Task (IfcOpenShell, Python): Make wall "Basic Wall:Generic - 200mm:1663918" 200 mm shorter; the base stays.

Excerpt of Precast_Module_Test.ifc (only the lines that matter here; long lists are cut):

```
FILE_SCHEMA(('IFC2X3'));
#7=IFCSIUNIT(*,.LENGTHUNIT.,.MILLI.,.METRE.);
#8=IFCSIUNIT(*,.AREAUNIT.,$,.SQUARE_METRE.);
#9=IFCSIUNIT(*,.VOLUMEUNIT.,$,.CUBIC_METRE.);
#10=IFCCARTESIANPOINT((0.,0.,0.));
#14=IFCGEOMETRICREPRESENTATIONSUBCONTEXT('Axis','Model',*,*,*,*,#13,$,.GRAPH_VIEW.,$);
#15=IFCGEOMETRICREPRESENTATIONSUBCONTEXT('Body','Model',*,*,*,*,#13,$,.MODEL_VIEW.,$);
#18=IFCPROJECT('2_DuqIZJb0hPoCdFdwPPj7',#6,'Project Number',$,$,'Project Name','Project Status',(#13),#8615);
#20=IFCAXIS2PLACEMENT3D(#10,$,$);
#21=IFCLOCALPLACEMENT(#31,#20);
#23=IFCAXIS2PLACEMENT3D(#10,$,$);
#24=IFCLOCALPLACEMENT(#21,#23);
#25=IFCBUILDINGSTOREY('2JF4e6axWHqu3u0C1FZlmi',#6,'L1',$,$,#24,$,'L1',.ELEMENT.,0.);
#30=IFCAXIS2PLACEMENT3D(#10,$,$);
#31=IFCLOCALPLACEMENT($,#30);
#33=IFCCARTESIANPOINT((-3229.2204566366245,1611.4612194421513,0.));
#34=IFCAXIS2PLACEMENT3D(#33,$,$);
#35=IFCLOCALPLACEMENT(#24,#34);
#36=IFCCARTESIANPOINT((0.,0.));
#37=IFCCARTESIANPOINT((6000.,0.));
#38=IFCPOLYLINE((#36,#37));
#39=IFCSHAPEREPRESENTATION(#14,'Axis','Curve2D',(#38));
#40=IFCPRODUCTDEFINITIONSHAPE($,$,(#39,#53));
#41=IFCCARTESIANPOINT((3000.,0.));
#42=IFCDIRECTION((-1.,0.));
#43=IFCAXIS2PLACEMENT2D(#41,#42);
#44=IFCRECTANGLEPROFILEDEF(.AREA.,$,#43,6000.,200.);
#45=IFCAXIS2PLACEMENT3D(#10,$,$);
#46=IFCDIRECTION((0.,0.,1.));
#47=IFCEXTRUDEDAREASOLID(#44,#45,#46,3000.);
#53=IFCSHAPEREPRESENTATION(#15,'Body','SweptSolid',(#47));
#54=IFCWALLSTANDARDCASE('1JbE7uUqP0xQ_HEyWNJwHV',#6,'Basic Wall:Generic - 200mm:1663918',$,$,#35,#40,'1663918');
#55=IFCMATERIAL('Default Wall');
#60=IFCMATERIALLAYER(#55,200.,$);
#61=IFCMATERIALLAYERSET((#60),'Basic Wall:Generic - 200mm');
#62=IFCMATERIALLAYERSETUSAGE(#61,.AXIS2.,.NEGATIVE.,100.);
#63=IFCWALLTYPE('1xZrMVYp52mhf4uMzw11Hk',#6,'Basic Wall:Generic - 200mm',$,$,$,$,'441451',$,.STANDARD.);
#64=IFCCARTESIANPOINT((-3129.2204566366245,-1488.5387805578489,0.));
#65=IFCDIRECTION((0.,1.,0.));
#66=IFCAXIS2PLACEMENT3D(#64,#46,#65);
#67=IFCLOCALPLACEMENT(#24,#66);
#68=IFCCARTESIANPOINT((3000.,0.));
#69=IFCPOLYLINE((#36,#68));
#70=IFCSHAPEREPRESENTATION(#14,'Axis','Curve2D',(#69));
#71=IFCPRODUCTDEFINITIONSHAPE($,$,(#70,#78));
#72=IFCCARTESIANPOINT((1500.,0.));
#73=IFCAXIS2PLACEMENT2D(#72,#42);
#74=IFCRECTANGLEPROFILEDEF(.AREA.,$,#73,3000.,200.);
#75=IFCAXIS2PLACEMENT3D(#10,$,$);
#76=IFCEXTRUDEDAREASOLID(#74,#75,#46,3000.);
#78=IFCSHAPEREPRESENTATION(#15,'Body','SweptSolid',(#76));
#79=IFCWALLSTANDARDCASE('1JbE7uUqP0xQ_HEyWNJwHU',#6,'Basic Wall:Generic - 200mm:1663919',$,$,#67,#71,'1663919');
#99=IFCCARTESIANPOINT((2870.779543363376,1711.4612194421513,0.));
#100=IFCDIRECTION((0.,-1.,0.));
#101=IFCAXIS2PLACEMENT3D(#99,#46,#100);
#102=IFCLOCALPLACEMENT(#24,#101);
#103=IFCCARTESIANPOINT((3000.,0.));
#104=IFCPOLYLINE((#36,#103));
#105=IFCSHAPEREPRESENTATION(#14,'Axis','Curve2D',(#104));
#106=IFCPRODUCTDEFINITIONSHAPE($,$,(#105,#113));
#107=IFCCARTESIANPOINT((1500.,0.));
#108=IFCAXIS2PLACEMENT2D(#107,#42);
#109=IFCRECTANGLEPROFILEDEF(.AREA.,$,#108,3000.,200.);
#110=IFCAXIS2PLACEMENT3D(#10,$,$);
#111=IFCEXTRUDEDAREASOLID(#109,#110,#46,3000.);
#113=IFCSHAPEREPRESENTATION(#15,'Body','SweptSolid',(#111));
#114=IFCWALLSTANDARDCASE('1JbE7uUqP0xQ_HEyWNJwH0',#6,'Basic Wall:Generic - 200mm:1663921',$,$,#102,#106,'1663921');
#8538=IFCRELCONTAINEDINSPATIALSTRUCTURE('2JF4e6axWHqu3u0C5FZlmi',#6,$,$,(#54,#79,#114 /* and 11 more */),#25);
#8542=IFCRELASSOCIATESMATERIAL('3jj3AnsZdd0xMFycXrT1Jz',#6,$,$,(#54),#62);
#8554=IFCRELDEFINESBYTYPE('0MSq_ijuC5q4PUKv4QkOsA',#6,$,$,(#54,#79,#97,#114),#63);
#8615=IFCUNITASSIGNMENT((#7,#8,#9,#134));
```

```python
import ifcopenshell
import ifcopenshell.geom
import ifcopenshell.util.representation
import ifcopenshell.util.shape
import ifcopenshell.util.unit

model = ifcopenshell.open("Precast_Module_Test.ifc")
unit_scale = ifcopenshell.util.unit.calculate_unit_scale(model)
settings = ifcopenshell.geom.settings()


def volume(element):
    """Net volume in cubic metres, openings subtracted."""
    shape = ifcopenshell.geom.create_shape(settings, element)
    return ifcopenshell.util.shape.get_volume(shape.geometry)


wall = model.by_guid("1JbE7uUqP0xQ_HEyWNJwHV")
before = volume(wall)

body = ifcopenshell.util.representation.get_representation(wall, "Model", "Body")
solid = body.Items[0]
old_height = solid.Depth
solid.Depth -= 0.2 / unit_scale
after = volume(wall)

print(f"height {old_height:g} -> {solid.Depth:g}, volume {before:.3f} -> {after:.3f} m3")

model.write("Precast_Module_Test-out.ifc")
```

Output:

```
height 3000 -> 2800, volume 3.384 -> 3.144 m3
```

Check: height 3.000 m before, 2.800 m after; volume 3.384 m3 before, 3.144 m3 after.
